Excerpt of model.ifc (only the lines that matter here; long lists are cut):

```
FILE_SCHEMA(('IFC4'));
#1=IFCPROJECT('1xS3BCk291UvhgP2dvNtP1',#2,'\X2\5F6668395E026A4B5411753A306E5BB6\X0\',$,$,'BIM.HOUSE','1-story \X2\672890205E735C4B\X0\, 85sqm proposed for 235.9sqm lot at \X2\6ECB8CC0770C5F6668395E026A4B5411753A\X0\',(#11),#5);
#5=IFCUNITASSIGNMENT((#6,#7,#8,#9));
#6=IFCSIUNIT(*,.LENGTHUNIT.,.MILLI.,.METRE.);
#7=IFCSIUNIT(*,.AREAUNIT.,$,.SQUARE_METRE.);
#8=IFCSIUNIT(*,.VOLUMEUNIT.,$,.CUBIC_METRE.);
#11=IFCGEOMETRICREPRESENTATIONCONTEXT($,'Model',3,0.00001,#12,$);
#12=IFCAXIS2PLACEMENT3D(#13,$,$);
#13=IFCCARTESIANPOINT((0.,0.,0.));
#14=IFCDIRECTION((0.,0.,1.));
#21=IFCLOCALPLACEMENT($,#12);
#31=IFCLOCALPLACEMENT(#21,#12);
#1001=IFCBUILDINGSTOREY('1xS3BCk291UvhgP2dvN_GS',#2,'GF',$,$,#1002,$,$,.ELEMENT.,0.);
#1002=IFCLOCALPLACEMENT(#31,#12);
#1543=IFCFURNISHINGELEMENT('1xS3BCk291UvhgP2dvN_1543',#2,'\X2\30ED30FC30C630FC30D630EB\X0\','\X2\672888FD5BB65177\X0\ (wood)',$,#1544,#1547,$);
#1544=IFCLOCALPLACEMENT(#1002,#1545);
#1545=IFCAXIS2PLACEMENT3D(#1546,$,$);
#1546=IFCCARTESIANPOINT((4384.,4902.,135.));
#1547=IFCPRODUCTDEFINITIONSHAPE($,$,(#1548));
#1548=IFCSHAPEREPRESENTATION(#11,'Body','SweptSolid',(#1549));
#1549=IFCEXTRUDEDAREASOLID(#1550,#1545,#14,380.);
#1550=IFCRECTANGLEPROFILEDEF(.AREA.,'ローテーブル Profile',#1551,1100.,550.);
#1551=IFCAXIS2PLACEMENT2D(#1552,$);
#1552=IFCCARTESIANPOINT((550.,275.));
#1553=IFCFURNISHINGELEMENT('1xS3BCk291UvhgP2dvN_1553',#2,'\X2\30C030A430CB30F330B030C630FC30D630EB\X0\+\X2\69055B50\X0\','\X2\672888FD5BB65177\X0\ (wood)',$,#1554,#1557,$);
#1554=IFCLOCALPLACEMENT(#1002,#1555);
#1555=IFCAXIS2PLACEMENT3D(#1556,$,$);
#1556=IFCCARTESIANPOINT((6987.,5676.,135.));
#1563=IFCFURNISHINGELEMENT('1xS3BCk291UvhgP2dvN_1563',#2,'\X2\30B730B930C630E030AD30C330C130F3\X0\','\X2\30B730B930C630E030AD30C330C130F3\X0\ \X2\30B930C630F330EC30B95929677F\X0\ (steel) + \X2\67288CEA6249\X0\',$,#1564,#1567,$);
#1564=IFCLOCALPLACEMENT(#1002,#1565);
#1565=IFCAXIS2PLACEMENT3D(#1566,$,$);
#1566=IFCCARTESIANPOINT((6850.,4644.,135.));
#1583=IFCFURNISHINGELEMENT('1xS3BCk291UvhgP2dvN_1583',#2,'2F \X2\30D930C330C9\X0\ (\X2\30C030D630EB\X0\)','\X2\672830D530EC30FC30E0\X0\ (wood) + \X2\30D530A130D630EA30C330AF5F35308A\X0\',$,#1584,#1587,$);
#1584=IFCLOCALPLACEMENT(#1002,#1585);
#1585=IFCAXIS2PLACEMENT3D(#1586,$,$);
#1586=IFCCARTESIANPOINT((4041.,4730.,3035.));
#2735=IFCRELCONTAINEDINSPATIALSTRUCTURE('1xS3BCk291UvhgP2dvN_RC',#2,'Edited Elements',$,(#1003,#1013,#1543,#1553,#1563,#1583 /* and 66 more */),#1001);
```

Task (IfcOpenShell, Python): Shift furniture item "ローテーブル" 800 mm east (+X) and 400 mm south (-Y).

```python
import ifcopenshell
import ifcopenshell.api.geometry
import ifcopenshell.util.placement
import ifcopenshell.util.unit

model = ifcopenshell.open("model.ifc")
unit_scale = ifcopenshell.util.unit.calculate_unit_scale(model)

item = model.by_id(1543)
matrix = ifcopenshell.util.placement.get_local_placement(item.ObjectPlacement)
matrix[0, 3] += 0.8 / unit_scale
matrix[1, 3] -= 0.4 / unit_scale
ifcopenshell.api.geometry.edit_object_placement(model, product=item, matrix=matrix, is_si=False)

print(ifcopenshell.util.placement.get_local_placement(item.ObjectPlacement).round(3) + 0.0)

model.write("model_edited.ifc")
```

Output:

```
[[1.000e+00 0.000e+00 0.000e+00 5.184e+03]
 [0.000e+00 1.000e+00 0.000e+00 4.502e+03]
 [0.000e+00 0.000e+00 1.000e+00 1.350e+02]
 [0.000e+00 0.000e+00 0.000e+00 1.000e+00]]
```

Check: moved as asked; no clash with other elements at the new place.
